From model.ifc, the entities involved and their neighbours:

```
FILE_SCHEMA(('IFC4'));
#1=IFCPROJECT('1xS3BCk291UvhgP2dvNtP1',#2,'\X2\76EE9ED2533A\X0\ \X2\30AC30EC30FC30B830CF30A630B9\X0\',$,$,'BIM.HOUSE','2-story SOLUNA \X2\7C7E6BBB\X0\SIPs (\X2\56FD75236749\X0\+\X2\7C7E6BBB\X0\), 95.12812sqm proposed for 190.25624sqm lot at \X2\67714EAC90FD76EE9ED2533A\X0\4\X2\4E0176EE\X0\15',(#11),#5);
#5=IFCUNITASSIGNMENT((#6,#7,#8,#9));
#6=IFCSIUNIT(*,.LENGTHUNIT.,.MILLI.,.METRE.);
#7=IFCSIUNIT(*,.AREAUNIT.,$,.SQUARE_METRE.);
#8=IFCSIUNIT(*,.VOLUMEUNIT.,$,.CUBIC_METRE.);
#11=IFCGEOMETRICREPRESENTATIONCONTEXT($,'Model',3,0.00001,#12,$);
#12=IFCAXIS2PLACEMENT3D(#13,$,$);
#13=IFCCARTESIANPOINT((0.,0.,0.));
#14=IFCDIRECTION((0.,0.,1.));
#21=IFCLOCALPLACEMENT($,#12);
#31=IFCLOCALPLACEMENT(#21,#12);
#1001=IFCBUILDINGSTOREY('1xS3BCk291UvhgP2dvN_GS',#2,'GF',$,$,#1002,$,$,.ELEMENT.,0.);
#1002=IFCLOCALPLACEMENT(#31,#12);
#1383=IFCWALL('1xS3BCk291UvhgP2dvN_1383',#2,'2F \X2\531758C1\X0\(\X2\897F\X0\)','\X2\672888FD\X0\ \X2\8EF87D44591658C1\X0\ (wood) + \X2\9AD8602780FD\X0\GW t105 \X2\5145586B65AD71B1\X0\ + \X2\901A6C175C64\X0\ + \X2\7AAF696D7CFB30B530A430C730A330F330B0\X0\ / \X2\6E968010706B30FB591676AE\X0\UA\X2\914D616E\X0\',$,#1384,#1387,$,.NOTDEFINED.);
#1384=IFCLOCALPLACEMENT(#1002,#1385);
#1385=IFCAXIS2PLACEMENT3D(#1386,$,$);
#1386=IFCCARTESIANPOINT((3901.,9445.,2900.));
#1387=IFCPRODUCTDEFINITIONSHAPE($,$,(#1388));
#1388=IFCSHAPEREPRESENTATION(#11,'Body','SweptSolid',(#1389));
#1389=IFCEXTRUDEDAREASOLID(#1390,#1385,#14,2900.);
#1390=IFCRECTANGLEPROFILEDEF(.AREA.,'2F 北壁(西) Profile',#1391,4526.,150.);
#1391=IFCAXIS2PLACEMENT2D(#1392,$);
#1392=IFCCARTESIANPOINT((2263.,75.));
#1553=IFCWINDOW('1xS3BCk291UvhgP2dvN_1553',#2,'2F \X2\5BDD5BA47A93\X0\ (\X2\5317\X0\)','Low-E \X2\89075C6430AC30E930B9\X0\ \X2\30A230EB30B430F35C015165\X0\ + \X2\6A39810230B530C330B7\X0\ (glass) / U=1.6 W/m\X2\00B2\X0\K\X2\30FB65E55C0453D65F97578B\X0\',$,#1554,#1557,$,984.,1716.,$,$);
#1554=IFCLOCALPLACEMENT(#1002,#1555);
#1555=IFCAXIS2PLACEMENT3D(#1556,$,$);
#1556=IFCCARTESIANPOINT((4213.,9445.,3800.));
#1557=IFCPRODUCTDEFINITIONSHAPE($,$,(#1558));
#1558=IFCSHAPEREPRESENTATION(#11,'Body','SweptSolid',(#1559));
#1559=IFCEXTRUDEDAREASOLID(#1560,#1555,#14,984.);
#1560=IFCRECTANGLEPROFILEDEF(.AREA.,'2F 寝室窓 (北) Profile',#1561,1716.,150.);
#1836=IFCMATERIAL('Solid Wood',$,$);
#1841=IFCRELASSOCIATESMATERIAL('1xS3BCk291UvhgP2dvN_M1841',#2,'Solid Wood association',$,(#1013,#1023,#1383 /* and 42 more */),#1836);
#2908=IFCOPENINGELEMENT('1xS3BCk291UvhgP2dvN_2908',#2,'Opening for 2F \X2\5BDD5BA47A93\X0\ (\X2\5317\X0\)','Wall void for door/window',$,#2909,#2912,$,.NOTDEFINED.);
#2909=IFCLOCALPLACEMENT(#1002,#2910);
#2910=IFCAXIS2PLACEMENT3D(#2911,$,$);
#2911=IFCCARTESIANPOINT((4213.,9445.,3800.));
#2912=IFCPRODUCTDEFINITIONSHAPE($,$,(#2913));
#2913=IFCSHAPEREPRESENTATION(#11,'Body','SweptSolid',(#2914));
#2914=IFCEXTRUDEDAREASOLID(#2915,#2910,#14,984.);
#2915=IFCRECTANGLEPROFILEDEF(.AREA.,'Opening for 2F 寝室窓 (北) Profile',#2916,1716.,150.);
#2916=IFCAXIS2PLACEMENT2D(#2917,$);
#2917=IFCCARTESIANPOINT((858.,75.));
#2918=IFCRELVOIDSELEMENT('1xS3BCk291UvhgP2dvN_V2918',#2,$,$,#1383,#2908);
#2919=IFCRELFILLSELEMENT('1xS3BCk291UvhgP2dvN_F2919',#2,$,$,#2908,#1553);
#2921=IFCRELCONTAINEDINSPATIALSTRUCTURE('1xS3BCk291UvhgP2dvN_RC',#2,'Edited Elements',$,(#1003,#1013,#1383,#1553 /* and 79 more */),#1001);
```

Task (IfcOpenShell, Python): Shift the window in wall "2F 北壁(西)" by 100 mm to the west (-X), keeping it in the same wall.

```python
import ifcopenshell
import ifcopenshell.api.geometry
import ifcopenshell.util.placement
import ifcopenshell.util.unit

model = ifcopenshell.open("model.ifc")
unit_scale = ifcopenshell.util.unit.calculate_unit_scale(model)

window = model.by_id(1553)
opening = window.FillsVoids[0].RelatingOpeningElement
wall = opening.VoidsElements[0].RelatingBuildingElement

wall_matrix = ifcopenshell.util.placement.get_local_placement(wall.ObjectPlacement)
shift = wall_matrix[:3, 0] * -0.1 / unit_scale
before = ifcopenshell.util.placement.get_local_placement(window.ObjectPlacement)[:3, 3].copy()

# The window is not placed relative to its opening, so move both.
for product in (opening, window):
    matrix = ifcopenshell.util.placement.get_local_placement(product.ObjectPlacement)
    matrix[:3, 3] += shift
    ifcopenshell.api.geometry.edit_object_placement(model, product=product, matrix=matrix, is_si=False)

after = ifcopenshell.util.placement.get_local_placement(window.ObjectPlacement)[:3, 3]
print("window moved by", (after - before).round(3) + 0.0)

model.write("model_rev.ifc")
```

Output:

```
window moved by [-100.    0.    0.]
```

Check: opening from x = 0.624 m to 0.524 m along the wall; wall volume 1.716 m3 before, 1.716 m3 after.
